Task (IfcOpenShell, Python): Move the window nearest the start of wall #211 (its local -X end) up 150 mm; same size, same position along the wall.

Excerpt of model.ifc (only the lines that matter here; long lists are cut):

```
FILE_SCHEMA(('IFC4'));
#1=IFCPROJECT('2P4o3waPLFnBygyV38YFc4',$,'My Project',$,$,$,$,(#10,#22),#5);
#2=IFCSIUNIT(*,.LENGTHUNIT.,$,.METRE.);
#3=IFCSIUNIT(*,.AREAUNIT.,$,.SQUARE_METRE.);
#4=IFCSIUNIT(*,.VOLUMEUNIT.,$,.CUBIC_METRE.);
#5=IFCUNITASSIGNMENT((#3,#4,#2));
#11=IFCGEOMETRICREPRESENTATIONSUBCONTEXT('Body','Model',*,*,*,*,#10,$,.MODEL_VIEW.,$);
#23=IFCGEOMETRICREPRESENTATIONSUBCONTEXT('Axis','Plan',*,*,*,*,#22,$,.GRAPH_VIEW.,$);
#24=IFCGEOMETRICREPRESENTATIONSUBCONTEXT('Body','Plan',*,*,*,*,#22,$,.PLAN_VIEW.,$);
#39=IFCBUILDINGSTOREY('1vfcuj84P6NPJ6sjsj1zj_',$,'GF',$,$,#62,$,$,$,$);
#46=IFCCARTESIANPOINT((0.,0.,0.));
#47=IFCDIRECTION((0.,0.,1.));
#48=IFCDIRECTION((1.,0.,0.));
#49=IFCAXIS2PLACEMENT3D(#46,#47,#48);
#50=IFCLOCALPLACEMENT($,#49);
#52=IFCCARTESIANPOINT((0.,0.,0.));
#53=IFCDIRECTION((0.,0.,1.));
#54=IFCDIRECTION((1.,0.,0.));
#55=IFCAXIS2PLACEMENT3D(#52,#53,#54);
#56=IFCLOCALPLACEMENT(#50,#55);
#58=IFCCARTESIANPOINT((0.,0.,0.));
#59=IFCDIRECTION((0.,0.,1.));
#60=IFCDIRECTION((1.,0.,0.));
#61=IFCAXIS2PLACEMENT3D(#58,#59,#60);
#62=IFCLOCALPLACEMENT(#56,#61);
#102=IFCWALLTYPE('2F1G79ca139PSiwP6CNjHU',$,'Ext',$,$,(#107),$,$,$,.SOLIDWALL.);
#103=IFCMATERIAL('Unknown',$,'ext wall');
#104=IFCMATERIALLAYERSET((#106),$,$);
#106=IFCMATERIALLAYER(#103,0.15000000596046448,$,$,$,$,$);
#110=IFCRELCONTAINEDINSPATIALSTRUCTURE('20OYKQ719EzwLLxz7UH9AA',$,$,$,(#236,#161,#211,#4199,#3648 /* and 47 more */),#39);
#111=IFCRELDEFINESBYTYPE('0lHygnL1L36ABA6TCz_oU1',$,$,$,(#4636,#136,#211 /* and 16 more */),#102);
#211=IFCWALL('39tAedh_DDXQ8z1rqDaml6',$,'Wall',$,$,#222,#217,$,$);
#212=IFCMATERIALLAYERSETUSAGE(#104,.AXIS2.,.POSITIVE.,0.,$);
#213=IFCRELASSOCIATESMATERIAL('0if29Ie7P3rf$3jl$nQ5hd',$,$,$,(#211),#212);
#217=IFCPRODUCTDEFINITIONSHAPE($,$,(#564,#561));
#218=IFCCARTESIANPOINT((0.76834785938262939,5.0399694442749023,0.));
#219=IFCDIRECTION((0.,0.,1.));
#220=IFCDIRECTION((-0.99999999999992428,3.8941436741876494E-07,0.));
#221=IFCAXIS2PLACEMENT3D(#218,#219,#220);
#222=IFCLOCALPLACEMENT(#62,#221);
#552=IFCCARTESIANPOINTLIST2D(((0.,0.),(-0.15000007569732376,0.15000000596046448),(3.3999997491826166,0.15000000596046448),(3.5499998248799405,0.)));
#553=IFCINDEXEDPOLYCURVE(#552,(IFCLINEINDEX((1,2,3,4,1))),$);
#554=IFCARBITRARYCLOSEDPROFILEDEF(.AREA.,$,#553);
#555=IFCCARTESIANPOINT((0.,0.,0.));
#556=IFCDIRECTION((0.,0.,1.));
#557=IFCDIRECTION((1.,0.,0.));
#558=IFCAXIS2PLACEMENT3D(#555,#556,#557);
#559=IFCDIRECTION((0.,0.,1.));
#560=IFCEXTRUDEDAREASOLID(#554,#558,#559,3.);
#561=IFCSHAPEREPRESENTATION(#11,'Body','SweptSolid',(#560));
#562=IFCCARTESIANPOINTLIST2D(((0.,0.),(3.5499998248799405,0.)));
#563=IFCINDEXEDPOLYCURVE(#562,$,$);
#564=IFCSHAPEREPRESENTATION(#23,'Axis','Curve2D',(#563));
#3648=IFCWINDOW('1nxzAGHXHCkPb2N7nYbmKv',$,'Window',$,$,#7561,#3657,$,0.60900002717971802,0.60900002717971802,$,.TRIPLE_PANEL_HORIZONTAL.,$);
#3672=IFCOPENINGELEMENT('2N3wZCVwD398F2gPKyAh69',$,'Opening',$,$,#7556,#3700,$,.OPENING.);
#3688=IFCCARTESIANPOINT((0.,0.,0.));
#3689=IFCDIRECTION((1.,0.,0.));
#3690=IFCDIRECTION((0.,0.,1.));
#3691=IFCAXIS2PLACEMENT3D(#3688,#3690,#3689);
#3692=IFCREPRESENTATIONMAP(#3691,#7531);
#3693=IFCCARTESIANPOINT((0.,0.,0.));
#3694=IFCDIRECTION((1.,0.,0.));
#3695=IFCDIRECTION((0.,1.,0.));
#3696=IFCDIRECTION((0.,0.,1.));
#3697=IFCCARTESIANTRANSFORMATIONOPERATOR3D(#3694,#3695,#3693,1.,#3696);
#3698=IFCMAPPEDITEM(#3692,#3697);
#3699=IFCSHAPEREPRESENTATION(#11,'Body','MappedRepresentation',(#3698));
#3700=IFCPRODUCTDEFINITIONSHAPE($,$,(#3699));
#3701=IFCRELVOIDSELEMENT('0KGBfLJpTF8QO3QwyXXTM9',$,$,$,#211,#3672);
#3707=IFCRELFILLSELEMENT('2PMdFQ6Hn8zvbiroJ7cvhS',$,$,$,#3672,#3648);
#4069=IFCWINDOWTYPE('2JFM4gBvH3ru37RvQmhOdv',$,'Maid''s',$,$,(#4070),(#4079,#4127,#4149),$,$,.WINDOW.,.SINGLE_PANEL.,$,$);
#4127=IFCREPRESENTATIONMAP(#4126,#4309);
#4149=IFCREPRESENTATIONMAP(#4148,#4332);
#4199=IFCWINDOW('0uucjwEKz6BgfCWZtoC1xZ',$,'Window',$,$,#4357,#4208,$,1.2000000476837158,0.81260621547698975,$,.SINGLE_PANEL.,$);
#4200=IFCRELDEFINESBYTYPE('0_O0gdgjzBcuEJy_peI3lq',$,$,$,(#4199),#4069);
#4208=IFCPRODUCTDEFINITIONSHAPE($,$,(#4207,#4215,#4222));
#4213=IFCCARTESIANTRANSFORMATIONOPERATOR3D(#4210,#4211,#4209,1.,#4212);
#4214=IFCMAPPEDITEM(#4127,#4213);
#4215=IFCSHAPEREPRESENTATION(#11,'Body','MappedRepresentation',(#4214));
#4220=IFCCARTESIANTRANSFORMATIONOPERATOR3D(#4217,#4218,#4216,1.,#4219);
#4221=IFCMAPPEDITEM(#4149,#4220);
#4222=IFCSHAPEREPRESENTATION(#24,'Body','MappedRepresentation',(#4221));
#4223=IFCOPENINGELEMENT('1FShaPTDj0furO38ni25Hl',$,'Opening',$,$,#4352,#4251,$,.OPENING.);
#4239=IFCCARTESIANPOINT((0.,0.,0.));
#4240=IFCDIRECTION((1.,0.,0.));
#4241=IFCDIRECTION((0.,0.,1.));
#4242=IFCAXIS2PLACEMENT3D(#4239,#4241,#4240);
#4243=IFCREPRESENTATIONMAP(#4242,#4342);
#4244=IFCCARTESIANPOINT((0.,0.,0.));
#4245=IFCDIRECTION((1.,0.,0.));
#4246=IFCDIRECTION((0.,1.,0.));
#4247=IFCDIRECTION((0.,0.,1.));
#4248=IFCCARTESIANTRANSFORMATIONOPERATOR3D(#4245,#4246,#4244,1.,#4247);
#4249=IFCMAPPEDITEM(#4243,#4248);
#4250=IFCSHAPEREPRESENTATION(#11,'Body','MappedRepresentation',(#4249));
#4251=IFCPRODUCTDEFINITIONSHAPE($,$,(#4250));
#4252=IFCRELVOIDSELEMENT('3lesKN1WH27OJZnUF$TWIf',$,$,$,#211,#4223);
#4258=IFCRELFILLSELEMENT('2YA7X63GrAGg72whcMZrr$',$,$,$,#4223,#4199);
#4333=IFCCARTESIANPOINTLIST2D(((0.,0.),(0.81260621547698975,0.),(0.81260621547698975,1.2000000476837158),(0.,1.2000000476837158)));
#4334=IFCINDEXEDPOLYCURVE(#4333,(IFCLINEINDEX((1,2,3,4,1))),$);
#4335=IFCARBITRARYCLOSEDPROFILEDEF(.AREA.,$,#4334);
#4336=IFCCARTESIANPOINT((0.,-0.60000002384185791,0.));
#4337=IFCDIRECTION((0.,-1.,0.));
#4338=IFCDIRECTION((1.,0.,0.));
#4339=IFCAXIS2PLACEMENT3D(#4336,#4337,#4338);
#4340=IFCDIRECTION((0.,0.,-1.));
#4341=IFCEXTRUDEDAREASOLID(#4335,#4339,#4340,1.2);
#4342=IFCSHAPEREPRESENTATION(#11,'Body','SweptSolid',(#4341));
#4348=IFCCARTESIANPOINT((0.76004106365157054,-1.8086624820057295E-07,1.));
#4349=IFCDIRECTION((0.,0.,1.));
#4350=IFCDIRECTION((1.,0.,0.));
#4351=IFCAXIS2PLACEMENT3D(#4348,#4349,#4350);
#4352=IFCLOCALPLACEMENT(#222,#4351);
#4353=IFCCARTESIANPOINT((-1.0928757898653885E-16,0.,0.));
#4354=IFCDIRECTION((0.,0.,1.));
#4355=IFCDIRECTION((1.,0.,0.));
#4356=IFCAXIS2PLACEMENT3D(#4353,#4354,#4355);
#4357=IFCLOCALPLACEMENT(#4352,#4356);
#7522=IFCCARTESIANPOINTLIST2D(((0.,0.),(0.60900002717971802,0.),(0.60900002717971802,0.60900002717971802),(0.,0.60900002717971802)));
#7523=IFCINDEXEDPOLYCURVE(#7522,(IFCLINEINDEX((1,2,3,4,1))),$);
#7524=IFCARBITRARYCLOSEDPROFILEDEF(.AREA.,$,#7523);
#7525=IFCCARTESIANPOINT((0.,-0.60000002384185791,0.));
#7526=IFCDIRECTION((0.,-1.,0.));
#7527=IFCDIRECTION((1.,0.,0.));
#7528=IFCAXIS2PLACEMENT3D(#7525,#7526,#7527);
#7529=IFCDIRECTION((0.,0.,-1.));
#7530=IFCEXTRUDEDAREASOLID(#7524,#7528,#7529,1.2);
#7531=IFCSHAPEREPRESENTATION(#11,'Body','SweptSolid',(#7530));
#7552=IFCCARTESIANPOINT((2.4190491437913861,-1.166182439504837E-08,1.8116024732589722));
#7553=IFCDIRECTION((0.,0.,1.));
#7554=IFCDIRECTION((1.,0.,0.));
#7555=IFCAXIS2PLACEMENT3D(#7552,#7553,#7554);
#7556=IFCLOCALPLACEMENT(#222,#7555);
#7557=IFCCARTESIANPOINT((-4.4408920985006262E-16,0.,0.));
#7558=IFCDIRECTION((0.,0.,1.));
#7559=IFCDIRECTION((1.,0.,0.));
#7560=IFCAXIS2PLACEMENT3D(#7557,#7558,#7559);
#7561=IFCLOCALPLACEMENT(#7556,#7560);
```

```python
import numpy as np
import ifcopenshell
import ifcopenshell.api.geometry
import ifcopenshell.util.placement
import ifcopenshell.util.unit

model = ifcopenshell.open("model.ifc")
unit_scale = ifcopenshell.util.unit.calculate_unit_scale(model)

window = model.by_guid("0uucjwEKz6BgfCWZtoC1xZ")
opening = window.FillsVoids[0].RelatingOpeningElement
dz = 0.15 / unit_scale

shift = np.array([0.0, 0.0, dz])
# The window is placed relative to its opening, so it follows when the opening moves.
matrix = ifcopenshell.util.placement.get_local_placement(opening.ObjectPlacement)
matrix[:3, 3] += shift
ifcopenshell.api.geometry.edit_object_placement(
    model, product=opening, matrix=matrix, is_si=False, should_transform_children=True
)

print(f"moved by {dz * unit_scale:+.3f} m")

model.write("model_edited.ifc")
```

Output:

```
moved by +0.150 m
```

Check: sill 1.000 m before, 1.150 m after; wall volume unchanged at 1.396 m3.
